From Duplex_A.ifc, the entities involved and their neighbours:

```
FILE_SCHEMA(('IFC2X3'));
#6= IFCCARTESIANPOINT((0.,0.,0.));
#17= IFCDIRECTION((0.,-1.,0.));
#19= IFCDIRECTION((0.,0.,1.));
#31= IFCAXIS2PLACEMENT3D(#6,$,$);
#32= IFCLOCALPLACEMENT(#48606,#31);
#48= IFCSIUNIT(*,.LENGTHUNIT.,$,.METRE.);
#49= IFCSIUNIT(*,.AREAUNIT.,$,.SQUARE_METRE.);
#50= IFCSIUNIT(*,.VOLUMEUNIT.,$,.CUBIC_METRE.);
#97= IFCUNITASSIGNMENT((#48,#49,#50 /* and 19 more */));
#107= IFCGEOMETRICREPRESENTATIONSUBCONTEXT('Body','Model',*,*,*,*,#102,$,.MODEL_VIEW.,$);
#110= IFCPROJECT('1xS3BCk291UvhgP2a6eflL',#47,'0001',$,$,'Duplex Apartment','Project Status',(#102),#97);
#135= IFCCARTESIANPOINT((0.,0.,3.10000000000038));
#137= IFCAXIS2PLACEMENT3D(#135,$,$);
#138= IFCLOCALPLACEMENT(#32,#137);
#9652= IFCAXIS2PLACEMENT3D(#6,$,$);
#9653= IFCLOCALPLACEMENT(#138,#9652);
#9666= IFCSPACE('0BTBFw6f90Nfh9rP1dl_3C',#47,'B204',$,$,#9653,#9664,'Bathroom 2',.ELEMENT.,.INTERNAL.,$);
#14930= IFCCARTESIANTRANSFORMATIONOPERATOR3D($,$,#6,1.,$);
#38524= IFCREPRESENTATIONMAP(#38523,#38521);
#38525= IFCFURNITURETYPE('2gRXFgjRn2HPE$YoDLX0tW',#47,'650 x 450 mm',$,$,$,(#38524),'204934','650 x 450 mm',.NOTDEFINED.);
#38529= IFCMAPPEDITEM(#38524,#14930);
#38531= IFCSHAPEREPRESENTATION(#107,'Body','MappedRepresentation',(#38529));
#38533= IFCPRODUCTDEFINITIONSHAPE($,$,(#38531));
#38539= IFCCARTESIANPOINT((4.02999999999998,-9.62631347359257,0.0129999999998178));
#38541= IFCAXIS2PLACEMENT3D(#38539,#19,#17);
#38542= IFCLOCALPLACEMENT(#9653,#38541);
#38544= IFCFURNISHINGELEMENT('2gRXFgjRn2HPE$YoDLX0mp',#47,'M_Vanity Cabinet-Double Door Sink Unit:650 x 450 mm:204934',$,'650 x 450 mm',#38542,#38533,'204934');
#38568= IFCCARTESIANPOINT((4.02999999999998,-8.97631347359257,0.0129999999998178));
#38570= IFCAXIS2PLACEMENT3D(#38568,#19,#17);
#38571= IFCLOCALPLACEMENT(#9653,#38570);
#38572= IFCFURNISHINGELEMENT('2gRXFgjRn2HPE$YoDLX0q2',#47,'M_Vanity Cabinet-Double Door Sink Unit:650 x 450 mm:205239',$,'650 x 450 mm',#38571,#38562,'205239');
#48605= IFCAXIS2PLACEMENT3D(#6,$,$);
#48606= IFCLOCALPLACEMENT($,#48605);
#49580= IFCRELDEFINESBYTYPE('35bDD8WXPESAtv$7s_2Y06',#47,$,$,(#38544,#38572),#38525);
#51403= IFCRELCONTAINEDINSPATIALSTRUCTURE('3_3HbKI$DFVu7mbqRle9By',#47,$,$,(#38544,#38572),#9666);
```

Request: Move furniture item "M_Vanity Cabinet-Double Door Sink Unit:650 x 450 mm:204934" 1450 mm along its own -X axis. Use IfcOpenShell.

```python
import ifcopenshell
import ifcopenshell.api.geometry
import ifcopenshell.util.placement
import ifcopenshell.util.unit

model = ifcopenshell.open("Duplex_A.ifc")
unit_scale = ifcopenshell.util.unit.calculate_unit_scale(model)

item = model.by_guid("2gRXFgjRn2HPE$YoDLX0mp")
matrix = ifcopenshell.util.placement.get_local_placement(item.ObjectPlacement)
matrix[:3, 3] -= matrix[:3, 0] * 1.45 / unit_scale
ifcopenshell.api.geometry.edit_object_placement(model, product=item, matrix=matrix, is_si=False)

print(ifcopenshell.util.placement.get_local_placement(item.ObjectPlacement).round(3) + 0.0)

model.write("Duplex_A_updated.ifc")
```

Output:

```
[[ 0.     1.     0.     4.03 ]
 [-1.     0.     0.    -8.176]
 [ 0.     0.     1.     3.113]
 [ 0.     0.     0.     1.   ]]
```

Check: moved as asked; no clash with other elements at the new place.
